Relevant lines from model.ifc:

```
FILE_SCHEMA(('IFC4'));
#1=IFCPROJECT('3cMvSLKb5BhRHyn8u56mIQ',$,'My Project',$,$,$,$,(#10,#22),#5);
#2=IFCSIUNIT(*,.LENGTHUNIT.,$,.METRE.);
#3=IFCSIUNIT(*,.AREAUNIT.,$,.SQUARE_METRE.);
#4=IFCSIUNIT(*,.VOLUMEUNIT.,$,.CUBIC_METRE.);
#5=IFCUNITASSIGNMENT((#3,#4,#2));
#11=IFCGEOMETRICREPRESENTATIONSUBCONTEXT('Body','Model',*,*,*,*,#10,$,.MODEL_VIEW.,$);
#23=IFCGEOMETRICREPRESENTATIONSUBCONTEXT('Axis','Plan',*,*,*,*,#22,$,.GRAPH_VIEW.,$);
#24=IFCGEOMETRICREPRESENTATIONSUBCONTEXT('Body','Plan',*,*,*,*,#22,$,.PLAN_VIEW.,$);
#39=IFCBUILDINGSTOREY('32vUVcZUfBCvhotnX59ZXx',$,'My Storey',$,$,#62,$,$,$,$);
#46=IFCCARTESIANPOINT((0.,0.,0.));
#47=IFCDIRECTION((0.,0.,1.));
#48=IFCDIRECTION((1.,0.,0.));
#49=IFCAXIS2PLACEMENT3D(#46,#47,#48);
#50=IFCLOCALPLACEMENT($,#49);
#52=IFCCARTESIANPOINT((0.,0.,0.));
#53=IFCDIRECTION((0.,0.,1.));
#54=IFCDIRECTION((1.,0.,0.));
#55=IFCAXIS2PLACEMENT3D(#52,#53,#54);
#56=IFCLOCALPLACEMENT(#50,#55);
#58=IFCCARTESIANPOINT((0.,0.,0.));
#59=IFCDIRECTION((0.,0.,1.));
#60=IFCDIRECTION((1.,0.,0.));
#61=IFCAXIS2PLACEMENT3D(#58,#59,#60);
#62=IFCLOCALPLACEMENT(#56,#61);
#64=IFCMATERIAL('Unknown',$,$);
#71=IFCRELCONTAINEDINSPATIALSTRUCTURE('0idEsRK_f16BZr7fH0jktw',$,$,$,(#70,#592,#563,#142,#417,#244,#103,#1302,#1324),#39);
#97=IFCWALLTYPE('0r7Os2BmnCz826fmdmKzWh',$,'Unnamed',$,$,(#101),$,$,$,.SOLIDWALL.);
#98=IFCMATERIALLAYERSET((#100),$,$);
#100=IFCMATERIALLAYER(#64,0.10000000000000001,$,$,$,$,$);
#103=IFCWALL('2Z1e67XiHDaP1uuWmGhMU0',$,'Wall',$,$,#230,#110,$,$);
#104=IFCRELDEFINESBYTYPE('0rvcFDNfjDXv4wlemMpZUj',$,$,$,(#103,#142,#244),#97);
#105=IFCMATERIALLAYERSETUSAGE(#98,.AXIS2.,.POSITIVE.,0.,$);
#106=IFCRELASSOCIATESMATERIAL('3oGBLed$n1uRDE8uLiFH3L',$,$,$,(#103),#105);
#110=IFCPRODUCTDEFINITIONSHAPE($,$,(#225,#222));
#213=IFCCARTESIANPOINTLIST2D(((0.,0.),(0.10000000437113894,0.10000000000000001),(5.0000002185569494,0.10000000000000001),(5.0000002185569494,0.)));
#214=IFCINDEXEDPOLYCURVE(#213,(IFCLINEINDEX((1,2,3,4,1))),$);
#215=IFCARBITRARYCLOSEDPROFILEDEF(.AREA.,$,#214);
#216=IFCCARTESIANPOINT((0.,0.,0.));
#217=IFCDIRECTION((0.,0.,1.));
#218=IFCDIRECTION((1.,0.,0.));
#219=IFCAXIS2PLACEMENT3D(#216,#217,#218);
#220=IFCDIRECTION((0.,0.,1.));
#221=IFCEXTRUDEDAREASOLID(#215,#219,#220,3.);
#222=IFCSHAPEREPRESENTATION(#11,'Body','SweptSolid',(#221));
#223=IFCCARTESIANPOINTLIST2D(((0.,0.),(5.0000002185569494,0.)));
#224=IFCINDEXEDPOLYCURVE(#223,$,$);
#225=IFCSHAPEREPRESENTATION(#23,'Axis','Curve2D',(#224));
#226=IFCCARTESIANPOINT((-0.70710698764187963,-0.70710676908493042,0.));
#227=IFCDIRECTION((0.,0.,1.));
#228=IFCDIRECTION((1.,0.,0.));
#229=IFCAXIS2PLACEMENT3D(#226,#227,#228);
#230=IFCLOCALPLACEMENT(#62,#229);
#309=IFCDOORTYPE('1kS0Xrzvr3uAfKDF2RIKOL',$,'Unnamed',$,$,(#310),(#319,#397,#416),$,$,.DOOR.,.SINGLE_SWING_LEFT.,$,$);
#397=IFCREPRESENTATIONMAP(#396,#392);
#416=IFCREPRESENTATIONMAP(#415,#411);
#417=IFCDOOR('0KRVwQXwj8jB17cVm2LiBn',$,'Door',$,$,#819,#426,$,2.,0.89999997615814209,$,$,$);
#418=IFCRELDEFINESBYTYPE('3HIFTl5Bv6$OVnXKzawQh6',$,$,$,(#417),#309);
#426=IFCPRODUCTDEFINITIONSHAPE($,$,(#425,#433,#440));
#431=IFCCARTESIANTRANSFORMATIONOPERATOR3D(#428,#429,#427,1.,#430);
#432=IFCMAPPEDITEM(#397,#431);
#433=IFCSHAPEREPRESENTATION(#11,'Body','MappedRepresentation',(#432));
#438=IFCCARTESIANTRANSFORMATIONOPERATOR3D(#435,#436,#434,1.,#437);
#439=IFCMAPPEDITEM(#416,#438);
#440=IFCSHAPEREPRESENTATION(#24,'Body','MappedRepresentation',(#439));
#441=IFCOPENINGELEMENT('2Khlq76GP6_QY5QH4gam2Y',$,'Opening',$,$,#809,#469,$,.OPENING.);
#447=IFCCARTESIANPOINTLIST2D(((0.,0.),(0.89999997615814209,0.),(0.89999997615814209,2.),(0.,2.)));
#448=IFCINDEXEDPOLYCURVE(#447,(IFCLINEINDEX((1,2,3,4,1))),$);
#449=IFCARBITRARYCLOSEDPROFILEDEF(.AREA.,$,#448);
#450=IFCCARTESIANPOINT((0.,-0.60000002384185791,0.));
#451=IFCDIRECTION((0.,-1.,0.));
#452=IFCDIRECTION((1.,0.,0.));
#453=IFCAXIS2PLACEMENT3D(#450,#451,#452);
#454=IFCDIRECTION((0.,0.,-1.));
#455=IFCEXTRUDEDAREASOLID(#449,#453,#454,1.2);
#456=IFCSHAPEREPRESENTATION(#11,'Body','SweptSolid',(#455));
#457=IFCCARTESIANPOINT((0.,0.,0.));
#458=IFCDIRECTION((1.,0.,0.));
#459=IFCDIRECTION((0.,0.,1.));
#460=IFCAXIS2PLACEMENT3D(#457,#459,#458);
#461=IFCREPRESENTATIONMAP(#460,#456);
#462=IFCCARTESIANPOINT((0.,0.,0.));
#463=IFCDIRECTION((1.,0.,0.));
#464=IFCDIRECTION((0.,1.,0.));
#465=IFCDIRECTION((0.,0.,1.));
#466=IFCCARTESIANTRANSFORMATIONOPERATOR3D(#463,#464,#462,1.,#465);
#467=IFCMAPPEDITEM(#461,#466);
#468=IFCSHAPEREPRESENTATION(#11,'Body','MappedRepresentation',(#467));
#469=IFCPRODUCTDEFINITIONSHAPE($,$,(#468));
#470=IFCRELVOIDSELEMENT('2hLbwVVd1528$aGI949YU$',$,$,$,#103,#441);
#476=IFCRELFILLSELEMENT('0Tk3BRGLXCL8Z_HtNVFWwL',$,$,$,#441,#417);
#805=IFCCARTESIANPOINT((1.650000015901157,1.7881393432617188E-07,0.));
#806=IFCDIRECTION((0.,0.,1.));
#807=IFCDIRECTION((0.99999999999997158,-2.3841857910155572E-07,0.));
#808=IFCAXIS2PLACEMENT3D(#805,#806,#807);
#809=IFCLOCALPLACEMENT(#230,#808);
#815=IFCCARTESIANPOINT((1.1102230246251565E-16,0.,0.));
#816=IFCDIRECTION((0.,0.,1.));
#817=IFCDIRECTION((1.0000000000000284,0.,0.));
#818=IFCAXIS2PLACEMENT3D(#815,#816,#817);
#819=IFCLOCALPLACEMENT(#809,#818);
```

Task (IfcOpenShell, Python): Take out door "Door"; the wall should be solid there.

```python
import ifcopenshell
import ifcopenshell.api.feature
import ifcopenshell.api.root
import ifcopenshell.geom
import ifcopenshell.util.shape

model = ifcopenshell.open("model.ifc")
settings = ifcopenshell.geom.settings()


def volume(element):
    """Net volume in cubic metres, openings subtracted."""
    shape = ifcopenshell.geom.create_shape(settings, element)
    return ifcopenshell.util.shape.get_volume(shape.geometry)


door = model.by_guid("0KRVwQXwj8jB17cVm2LiBn")
opening = door.FillsVoids[0].RelatingOpeningElement
wall = opening.VoidsElements[0].RelatingBuildingElement
before = volume(wall)

ifcopenshell.api.root.remove_product(model, product=door)
ifcopenshell.api.feature.remove_feature(model, feature=opening)

after = volume(wall)

print(f"wall volume {before:.3f} -> {after:.3f} m3")

model.write("model_updated.ifc")
```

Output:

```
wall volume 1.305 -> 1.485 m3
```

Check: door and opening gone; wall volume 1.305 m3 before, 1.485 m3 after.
